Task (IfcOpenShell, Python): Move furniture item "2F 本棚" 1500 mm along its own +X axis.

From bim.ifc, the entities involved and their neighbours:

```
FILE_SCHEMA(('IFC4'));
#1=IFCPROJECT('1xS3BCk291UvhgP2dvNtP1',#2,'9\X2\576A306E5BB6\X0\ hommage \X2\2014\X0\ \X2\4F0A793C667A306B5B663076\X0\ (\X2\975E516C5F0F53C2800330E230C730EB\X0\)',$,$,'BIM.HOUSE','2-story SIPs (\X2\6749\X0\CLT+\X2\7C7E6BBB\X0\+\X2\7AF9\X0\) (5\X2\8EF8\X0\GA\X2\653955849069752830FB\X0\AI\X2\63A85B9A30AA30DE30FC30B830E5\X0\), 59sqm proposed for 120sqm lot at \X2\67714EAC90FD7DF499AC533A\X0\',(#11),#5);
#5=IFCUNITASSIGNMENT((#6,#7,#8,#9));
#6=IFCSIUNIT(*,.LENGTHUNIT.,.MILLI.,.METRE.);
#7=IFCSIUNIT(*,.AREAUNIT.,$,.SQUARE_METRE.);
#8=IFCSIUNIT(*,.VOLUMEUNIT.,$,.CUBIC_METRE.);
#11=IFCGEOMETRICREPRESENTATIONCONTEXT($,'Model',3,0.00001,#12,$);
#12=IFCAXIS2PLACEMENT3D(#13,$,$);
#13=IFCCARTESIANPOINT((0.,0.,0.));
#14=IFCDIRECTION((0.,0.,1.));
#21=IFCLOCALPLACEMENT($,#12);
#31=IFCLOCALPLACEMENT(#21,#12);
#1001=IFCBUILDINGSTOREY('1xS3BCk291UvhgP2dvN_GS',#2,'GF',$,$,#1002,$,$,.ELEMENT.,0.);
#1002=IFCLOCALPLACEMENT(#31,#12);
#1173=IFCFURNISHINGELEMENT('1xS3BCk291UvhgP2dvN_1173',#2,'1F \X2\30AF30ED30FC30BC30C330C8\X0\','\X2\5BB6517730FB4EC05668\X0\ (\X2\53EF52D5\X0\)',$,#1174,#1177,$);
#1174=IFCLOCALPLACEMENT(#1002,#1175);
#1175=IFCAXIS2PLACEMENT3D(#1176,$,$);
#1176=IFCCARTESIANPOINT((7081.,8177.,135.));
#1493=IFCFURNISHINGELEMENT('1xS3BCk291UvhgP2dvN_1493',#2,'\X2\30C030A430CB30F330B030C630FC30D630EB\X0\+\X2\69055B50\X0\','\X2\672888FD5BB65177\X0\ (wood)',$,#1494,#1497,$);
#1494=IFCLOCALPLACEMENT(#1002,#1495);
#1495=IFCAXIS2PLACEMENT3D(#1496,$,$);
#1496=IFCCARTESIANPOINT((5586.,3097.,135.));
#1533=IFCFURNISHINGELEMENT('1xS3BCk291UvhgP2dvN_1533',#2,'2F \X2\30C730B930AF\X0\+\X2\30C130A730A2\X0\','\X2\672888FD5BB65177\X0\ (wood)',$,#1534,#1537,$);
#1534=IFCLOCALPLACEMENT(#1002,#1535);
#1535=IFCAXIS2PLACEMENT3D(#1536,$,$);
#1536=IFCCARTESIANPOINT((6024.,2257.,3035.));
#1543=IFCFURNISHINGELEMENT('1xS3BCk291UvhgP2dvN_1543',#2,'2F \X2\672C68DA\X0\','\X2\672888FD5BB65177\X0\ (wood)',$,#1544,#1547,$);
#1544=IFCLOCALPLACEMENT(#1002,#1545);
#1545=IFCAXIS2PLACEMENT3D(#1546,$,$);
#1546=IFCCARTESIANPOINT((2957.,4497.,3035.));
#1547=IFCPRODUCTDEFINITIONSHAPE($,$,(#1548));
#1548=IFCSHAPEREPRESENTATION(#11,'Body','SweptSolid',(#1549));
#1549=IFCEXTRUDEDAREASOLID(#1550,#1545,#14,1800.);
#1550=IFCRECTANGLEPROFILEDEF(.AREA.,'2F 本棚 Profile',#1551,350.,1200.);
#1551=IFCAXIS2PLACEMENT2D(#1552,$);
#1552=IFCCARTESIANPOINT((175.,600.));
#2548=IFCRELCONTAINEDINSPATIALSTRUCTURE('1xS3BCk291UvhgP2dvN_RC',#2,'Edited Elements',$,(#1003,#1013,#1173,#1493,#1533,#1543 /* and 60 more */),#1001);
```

```python
import ifcopenshell
import ifcopenshell.api.geometry
import ifcopenshell.util.placement
import ifcopenshell.util.unit

model = ifcopenshell.open("bim.ifc")
unit_scale = ifcopenshell.util.unit.calculate_unit_scale(model)

item = model.by_guid("1xS3BCk291UvhgP2dvN_1543")
matrix = ifcopenshell.util.placement.get_local_placement(item.ObjectPlacement)
matrix[:3, 3] += matrix[:3, 0] * 1.5 / unit_scale
ifcopenshell.api.geometry.edit_object_placement(model, product=item, matrix=matrix, is_si=False)

print(ifcopenshell.util.placement.get_local_placement(item.ObjectPlacement).round(3) + 0.0)

model.write("bim_rev.ifc")
```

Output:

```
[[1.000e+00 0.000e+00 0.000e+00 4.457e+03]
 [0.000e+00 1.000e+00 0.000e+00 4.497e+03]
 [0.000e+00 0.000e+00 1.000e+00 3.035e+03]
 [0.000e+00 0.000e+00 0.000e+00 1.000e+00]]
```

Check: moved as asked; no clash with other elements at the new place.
